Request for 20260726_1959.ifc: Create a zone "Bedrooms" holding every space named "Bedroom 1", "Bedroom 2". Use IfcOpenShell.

First a look at what the model holds.

```python
import ifcopenshell

model = ifcopenshell.open("20260726_1959.ifc")
print(model.schema)
seen = {}
for space in model.by_type("IfcSpace"):
    seen[space.LongName] = seen.get(space.LongName, 0) + 1
for name, count in sorted(seen.items(), key=str):
    print(count, "x", name)
print("zones:", [z.Name for z in model.by_type("IfcZone")][:20])
```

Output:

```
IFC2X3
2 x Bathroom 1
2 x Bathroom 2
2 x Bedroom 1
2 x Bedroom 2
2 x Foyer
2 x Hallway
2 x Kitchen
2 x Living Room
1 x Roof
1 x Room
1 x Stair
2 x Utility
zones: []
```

```python
import ifcopenshell
import ifcopenshell.api.group
import ifcopenshell.api.root

model = ifcopenshell.open("20260726_1959.ifc")

names = {"Bedroom 1", "Bedroom 2"}
spaces = [s for s in model.by_type("IfcSpace") if s.LongName in names]

zone = ifcopenshell.api.root.create_entity(model, ifc_class="IfcZone", name="Bedrooms")
ifcopenshell.api.group.assign_group(model, products=spaces, group=zone)
print(len(spaces), "spaces in", zone.Name)

model.write("20260726_1959_edited.ifc")
```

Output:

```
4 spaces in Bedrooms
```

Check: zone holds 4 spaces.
